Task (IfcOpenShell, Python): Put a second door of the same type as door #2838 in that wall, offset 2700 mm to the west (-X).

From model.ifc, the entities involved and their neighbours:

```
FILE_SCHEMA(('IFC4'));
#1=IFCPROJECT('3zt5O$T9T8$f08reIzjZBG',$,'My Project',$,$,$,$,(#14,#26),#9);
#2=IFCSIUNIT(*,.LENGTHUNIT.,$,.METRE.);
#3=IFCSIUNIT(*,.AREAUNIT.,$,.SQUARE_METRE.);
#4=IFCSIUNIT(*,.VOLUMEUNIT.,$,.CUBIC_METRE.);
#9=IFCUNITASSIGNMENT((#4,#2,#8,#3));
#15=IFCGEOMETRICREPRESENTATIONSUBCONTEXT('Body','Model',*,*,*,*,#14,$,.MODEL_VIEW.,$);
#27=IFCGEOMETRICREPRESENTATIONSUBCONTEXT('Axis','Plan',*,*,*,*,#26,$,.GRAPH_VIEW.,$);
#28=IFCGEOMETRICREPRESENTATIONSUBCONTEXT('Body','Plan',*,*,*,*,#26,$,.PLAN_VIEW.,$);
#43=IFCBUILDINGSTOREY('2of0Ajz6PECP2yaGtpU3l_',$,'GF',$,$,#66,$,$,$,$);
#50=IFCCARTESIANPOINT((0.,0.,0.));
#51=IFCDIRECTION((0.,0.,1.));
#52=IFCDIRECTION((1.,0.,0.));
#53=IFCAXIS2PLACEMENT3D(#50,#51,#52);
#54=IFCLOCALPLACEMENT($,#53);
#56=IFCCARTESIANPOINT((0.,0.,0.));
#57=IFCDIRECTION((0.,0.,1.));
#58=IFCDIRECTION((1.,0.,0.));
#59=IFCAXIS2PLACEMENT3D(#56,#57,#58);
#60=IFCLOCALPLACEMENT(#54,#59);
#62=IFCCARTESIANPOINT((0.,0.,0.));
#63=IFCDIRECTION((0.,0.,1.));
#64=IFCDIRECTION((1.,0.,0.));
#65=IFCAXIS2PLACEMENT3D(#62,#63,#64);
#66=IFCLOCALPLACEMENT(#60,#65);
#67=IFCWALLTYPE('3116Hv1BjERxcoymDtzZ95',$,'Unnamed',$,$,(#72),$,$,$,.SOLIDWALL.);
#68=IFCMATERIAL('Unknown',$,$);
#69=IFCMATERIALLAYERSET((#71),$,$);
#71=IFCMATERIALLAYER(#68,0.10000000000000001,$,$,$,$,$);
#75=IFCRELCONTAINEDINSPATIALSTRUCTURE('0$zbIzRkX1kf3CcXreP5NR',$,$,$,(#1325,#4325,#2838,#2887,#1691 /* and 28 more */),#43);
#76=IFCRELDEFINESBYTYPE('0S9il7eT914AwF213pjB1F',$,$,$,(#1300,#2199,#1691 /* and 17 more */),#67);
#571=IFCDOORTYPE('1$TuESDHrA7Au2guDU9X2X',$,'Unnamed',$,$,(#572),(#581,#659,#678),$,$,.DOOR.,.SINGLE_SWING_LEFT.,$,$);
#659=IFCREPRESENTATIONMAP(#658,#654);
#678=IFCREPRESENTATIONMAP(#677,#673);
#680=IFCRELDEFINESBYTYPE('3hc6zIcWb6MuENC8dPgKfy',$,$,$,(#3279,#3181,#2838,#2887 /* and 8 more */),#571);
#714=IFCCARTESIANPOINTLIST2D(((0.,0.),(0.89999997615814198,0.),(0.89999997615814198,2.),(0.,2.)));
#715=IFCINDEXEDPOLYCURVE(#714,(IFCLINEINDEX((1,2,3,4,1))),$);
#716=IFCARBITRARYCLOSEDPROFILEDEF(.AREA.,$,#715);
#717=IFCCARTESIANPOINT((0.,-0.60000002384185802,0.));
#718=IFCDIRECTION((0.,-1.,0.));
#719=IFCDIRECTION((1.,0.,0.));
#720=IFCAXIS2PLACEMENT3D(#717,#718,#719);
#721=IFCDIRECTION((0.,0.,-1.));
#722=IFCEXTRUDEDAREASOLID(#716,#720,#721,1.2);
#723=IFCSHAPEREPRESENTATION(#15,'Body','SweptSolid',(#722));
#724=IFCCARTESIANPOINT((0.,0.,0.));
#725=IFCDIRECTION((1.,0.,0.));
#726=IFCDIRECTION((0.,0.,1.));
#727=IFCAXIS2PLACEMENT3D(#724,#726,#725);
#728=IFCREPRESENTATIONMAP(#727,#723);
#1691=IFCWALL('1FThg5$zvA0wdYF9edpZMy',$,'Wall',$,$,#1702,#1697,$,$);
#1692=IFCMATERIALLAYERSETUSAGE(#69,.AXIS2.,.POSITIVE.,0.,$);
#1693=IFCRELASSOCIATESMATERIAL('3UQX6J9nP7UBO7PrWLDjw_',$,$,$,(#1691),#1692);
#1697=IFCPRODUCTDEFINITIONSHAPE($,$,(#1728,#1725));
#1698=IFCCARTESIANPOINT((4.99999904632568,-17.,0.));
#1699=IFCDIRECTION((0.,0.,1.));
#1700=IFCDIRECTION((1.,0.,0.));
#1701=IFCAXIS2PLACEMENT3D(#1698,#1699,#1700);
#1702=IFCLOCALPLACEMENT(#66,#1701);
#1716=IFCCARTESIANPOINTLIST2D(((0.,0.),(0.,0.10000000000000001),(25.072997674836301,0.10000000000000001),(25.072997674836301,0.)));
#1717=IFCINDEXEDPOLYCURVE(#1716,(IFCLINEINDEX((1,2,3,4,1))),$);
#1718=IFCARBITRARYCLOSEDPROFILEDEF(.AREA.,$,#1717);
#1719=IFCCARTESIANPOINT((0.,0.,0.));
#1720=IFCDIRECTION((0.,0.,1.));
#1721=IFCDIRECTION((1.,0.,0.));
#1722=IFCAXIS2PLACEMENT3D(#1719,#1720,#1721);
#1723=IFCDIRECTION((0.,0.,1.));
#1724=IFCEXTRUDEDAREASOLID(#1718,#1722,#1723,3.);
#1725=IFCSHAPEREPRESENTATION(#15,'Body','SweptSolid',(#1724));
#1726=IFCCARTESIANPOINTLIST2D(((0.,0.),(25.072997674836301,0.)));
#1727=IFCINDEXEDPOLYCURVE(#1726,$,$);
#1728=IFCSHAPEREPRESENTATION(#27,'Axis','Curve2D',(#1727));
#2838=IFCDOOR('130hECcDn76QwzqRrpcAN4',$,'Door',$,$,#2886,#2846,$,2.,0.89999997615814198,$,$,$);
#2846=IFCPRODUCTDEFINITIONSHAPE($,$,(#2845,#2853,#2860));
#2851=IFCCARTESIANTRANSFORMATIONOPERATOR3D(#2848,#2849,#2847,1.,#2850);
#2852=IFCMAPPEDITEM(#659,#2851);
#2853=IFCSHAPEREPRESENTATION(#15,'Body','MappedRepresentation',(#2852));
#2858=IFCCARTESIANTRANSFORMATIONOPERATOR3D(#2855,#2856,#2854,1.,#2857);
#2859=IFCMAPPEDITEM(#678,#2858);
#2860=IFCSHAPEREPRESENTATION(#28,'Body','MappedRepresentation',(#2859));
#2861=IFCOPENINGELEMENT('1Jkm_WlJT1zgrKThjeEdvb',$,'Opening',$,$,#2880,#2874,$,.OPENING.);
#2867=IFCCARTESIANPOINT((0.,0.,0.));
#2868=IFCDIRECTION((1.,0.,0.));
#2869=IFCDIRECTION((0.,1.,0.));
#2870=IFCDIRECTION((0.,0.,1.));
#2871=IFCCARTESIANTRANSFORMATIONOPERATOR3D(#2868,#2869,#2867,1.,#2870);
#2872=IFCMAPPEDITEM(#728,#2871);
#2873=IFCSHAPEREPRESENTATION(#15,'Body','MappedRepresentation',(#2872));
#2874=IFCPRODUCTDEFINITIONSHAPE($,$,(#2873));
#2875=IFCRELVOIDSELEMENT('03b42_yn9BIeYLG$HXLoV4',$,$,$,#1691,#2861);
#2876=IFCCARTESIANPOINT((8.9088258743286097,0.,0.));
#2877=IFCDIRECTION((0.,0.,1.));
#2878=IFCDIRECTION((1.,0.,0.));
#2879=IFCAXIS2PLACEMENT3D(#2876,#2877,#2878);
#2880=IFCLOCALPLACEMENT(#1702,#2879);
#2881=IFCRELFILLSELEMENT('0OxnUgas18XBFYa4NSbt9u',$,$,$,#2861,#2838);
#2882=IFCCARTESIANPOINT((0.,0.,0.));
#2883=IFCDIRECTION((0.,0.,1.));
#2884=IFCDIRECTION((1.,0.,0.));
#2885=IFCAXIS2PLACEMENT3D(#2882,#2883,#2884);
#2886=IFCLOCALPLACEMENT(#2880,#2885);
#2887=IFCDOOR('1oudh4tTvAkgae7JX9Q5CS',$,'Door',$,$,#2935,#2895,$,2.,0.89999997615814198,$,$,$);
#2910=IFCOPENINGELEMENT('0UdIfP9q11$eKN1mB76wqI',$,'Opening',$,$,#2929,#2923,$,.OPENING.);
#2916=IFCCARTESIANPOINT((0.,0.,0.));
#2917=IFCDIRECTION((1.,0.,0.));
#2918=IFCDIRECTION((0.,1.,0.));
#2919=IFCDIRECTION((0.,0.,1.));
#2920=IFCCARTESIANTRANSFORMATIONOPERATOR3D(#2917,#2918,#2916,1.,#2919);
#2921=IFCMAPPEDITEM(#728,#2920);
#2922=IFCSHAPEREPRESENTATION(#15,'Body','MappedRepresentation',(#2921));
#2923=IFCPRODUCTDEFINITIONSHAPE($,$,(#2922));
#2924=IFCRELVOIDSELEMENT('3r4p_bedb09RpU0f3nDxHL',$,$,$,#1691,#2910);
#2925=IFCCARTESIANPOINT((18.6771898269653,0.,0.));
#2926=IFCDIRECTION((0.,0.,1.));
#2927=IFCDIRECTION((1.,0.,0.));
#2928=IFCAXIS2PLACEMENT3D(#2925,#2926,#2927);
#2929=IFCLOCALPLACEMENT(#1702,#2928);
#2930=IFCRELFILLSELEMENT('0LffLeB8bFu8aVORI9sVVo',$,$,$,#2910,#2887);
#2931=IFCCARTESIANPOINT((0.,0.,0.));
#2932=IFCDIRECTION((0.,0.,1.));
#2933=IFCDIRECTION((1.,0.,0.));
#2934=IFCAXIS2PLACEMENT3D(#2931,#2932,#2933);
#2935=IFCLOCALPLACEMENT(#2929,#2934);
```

```python
import ifcopenshell
import ifcopenshell.api.feature
import ifcopenshell.api.geometry
import ifcopenshell.api.root
import ifcopenshell.geom
import ifcopenshell.util.element
import ifcopenshell.util.placement
import ifcopenshell.util.shape
import ifcopenshell.util.unit

model = ifcopenshell.open("model.ifc")
unit_scale = ifcopenshell.util.unit.calculate_unit_scale(model)
settings = ifcopenshell.geom.settings()


def volume(element):
    """Net volume in cubic metres, openings subtracted."""
    shape = ifcopenshell.geom.create_shape(settings, element)
    return ifcopenshell.util.shape.get_volume(shape.geometry)


door = model.by_guid("130hECcDn76QwzqRrpcAN4")
opening = door.FillsVoids[0].RelatingOpeningElement
wall = opening.VoidsElements[0].RelatingBuildingElement
before = volume(wall)
shift = ifcopenshell.util.placement.get_local_placement(wall.ObjectPlacement)[:3, 0] * -2.7 / unit_scale

# copy_class copies the void relationship, type, container and properties, but no geometry.
new_opening = ifcopenshell.api.root.copy_class(model, product=opening)
new_opening.Representation = ifcopenshell.util.element.copy_deep(
    model, opening.Representation, exclude=["IfcGeometricRepresentationContext", "IfcRepresentationMap"]
)
new_door = ifcopenshell.api.root.copy_class(model, product=door)
new_door.Representation = ifcopenshell.util.element.copy_deep(
    model, door.Representation, exclude=["IfcGeometricRepresentationContext", "IfcRepresentationMap"]
)
ifcopenshell.api.feature.add_filling(model, opening=new_opening, element=new_door)

for old, new in ((opening, new_opening), (door, new_door)):
    matrix = ifcopenshell.util.placement.get_local_placement(old.ObjectPlacement)
    matrix[:3, 3] += shift
    ifcopenshell.api.geometry.edit_object_placement(model, product=new, matrix=matrix, is_si=False)

after = volume(wall)

print(f"wall volume {before:.3f} -> {after:.3f} m3")

model.write("model-out.ifc")
```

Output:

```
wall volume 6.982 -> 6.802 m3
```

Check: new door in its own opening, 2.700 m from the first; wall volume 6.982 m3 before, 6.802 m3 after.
